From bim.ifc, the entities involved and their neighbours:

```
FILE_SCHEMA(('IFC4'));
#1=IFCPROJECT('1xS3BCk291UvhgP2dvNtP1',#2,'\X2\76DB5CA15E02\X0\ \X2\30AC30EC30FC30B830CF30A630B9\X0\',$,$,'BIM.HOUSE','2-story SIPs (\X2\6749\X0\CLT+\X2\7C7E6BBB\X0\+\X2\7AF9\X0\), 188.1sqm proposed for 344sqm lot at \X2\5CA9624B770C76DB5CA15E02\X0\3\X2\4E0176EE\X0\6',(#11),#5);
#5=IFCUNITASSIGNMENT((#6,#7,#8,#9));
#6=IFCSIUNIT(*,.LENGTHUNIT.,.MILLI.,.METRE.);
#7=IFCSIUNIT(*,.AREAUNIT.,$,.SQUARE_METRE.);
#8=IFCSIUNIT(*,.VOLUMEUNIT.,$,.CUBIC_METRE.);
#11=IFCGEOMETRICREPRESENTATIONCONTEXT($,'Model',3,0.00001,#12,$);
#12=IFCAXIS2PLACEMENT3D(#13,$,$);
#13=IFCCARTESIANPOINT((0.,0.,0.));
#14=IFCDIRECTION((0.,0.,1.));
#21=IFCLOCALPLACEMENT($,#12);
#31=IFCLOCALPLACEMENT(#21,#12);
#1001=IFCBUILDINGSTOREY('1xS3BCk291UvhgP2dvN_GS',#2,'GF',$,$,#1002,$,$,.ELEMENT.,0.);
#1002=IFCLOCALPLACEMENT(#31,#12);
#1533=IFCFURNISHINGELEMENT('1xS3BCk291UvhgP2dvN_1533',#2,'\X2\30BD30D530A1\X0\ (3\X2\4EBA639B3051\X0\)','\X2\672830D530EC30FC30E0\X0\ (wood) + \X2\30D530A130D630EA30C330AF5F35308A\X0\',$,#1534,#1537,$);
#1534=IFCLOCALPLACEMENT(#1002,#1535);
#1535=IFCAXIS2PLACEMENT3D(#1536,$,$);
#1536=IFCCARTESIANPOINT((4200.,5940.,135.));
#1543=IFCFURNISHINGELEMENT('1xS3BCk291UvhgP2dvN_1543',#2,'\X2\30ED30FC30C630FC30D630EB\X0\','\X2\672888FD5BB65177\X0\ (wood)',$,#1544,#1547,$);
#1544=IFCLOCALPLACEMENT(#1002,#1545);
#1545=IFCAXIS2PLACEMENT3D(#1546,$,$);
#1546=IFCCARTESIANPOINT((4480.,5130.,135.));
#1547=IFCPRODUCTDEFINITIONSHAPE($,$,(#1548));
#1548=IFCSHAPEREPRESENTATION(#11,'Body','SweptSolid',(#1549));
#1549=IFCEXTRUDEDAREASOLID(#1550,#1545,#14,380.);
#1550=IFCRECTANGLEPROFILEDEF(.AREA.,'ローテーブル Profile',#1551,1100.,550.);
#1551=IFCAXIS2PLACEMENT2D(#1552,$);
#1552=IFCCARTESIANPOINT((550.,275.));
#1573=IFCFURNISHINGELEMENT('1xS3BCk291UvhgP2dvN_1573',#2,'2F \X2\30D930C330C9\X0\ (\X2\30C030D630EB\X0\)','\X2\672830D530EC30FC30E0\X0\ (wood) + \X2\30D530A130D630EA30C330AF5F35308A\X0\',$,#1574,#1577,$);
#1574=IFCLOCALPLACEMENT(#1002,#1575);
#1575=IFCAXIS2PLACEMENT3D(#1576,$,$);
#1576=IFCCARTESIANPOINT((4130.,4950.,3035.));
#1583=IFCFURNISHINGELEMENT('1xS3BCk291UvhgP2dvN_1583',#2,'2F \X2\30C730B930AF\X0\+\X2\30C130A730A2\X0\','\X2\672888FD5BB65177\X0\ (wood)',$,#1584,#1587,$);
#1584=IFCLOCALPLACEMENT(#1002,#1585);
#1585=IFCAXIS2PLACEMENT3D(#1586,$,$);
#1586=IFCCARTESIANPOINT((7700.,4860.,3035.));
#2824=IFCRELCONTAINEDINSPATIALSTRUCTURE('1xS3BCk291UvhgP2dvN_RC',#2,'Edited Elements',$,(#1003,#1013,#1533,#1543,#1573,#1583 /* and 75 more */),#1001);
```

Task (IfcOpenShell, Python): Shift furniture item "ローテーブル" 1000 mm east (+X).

```python
import ifcopenshell
import ifcopenshell.api.geometry
import ifcopenshell.util.placement
import ifcopenshell.util.unit

model = ifcopenshell.open("bim.ifc")
unit_scale = ifcopenshell.util.unit.calculate_unit_scale(model)

item = model.by_id(1543)
matrix = ifcopenshell.util.placement.get_local_placement(item.ObjectPlacement)
matrix[0, 3] += 1 / unit_scale
ifcopenshell.api.geometry.edit_object_placement(model, product=item, matrix=matrix, is_si=False)

print(ifcopenshell.util.placement.get_local_placement(item.ObjectPlacement).round(3) + 0.0)

model.write("bim_rev.ifc")
```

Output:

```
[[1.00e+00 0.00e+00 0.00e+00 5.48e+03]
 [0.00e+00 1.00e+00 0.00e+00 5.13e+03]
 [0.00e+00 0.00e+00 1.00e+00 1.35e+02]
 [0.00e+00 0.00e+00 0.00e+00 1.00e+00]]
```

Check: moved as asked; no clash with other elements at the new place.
